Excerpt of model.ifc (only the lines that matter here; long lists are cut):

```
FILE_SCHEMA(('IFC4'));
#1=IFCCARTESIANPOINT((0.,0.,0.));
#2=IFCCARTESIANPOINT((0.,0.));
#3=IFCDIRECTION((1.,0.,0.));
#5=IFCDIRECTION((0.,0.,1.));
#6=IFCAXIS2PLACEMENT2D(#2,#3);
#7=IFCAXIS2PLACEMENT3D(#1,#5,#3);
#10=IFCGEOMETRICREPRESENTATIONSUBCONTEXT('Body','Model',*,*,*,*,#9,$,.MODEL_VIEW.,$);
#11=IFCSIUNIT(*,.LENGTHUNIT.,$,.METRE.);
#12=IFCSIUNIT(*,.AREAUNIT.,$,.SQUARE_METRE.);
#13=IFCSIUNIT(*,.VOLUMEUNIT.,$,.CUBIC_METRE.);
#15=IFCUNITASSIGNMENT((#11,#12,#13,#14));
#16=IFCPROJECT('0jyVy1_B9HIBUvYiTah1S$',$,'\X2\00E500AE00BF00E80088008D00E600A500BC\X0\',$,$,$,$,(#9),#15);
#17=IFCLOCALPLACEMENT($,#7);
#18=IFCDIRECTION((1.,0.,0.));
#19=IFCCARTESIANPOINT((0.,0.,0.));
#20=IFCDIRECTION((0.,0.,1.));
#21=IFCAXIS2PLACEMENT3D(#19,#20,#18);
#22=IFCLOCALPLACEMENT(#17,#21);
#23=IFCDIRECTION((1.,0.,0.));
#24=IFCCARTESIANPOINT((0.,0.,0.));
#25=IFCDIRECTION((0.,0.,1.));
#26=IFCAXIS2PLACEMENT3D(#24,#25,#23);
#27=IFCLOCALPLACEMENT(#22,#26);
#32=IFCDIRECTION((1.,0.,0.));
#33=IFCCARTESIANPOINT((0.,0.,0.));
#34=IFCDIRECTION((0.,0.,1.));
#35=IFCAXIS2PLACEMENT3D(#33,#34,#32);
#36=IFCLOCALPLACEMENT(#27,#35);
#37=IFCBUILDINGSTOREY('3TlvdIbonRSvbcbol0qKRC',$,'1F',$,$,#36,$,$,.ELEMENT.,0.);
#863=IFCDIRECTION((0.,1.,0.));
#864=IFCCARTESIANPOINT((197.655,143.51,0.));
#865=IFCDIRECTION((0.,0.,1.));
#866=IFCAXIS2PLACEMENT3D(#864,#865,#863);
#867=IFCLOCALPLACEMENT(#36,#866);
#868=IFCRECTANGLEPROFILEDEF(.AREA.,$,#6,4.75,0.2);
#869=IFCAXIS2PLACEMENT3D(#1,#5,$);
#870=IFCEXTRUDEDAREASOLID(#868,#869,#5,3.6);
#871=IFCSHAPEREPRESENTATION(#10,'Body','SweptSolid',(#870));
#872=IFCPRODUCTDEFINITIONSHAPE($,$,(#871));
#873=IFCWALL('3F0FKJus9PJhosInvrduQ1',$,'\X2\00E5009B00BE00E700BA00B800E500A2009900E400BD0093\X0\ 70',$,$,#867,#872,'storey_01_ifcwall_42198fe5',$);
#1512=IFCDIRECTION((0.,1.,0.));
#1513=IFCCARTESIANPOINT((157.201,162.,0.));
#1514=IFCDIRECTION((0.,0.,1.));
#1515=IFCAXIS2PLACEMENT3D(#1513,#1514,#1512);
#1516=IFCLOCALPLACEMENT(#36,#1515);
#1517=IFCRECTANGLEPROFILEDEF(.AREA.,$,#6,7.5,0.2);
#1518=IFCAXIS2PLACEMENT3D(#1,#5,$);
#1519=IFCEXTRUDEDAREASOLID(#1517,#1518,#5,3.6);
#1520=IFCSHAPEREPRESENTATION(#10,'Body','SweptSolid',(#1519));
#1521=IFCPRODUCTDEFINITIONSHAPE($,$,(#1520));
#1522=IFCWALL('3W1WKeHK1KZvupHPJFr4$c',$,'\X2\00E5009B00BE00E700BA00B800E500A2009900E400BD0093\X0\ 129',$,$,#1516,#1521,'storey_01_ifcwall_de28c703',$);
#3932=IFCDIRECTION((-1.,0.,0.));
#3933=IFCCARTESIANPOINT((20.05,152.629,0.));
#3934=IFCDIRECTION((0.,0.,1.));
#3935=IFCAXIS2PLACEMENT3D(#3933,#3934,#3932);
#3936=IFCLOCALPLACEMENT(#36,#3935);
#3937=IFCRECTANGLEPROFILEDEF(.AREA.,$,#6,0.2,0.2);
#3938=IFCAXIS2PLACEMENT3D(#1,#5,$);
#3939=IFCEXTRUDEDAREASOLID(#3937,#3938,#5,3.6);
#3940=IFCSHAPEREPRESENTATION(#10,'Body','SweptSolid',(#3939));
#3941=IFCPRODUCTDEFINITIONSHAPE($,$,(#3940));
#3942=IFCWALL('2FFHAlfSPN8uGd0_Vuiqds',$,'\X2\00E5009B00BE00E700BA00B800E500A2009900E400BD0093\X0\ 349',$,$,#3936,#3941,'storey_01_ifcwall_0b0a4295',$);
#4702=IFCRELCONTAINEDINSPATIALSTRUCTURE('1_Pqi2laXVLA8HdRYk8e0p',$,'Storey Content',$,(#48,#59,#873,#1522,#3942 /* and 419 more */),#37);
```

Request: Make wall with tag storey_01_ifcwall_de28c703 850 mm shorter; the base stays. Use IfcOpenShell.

```python
import ifcopenshell
import ifcopenshell.geom
import ifcopenshell.util.representation
import ifcopenshell.util.shape

model = ifcopenshell.open("model.ifc")
settings = ifcopenshell.geom.settings()


def volume(element):
    """Net volume in cubic metres, openings subtracted."""
    shape = ifcopenshell.geom.create_shape(settings, element)
    return ifcopenshell.util.shape.get_volume(shape.geometry)


wall = model.by_guid("3W1WKeHK1KZvupHPJFr4$c")
before = volume(wall)

body = ifcopenshell.util.representation.get_representation(wall, "Model", "Body")
solid = body.Items[0]
old_height = solid.Depth
solid.Depth -= 0.85
after = volume(wall)

print(f"height {old_height:g} -> {solid.Depth:g}, volume {before:.3f} -> {after:.3f} m3")

model.write("model_updated.ifc")
```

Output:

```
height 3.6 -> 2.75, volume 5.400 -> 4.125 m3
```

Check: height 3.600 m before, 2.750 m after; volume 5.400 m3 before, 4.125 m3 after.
